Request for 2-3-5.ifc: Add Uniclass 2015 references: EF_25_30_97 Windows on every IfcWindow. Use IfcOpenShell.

First a look at what the model holds.

```python
import ifcopenshell

model = ifcopenshell.open("2-3-5.ifc")
print(model.schema)
print("classifications:", [c.Name for c in model.by_type("IfcClassification")])
for ifc_class in ("IfcDoor", "IfcRoof", "IfcStair", "IfcWall", "IfcWindow"):
    print(ifc_class, len(model.by_type(ifc_class)))
```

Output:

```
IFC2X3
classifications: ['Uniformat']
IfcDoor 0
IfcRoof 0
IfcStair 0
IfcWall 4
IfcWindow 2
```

```python
import ifcopenshell
import ifcopenshell.api.classification

model = ifcopenshell.open("2-3-5.ifc")

# IFC2X3 requires Source and Edition and has no link from the project to the system.
system = model.create_entity("IfcClassification", Source="NBS", Edition="2015", Name="Uniclass 2015")

codes = {
    "IfcWindow": ("EF_25_30_97", "Windows"),
}
for ifc_class, (code, name) in codes.items():
    products = model.by_type(ifc_class)
    ifcopenshell.api.classification.add_reference(
        model, products=products, classification=system, identification=code, name=name
    )
    print(code, len(products))

model.write("2-3-5_edited.ifc")
```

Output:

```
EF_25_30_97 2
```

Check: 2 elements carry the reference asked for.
